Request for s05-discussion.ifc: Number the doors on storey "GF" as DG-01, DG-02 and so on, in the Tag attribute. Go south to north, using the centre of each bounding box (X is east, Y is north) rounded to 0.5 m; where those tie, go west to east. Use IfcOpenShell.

First a look at what the model holds.

```python
import ifcopenshell
import ifcopenshell.util.element
import ifcopenshell.util.placement

model = ifcopenshell.open("s05-discussion.ifc")
print(model.schema)
storey = next(s for s in model.by_type("IfcBuildingStorey") if s.Name == "GF")
doors = [e for e in ifcopenshell.util.element.get_decomposition(storey) if e.is_a("IfcDoor")]
for e in sorted(doors, key=lambda e: e.id()):
    origin = ifcopenshell.util.placement.get_local_placement(e.ObjectPlacement)[:3, 3]
    print(e.id(), e.Tag, e.Name, origin.round(2) + 0.0, sep=" | ")
```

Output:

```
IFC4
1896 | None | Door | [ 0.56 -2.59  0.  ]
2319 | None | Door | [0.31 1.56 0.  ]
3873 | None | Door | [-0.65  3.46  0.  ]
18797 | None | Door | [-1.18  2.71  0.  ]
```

```python
import ifcopenshell
import ifcopenshell.geom
import ifcopenshell.util.element
import ifcopenshell.util.shape

model = ifcopenshell.open("s05-discussion.ifc")
settings = ifcopenshell.geom.settings()
settings.set("use-world-coords", True)


def centre(element):
    shape = ifcopenshell.geom.create_shape(settings, element)
    return ifcopenshell.util.shape.get_bbox_centroid(shape.geometry)


storey = next(s for s in model.by_type("IfcBuildingStorey") if s.Name == "GF")
doors = [e for e in ifcopenshell.util.element.get_decomposition(storey) if e.is_a("IfcDoor")]

# Insertion points can sit at a corner or the storey origin, so sort by the geometry (in metres).
centres = {e: centre(e) for e in doors}
doors.sort(key=lambda e: (round(centres[e][1] / 0.5), centres[e][0]))

for i, e in enumerate(doors, start=1):
    number = f"DG-{i:02d}"
    e.Tag = number
    print(e.id(), number)

model.write("s05-discussion_edited.ifc")
```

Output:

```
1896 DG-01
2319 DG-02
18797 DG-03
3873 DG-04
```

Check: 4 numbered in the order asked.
